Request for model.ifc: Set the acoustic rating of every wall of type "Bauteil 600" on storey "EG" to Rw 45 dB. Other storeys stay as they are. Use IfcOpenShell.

First a look at what the model holds.

```python
import ifcopenshell
import ifcopenshell.util.element

model = ifcopenshell.open("model.ifc")
print(model.schema)
storey = next(s for s in model.by_type("IfcBuildingStorey") if s.Name == "EG")
walls = [e for e in ifcopenshell.util.element.get_decomposition(storey) if e.is_a("IfcWall")]
seen = {}
for e in walls:
    element_type = ifcopenshell.util.element.get_type(e)
    key = (element_type.Name if element_type != e and element_type else None, ifcopenshell.util.element.get_pset(e, "Pset_WallCommon", "AcousticRating"))
    seen[key] = seen.get(key, 0) + 1
for (name, value), count in sorted(seen.items(), key=str):
    print(count, "x", name, "|", value)
```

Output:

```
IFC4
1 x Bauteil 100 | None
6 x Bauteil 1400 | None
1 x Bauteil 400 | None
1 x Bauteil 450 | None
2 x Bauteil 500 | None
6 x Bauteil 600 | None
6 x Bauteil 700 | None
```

```python
import ifcopenshell
import ifcopenshell.api.pset
import ifcopenshell.util.element

model = ifcopenshell.open("model.ifc")

storey = next(s for s in model.by_type("IfcBuildingStorey") if s.Name == "EG")
walls = [e for e in ifcopenshell.util.element.get_decomposition(storey) if e.is_a("IfcWall")]

count = 0
for e in walls:
    element_type = ifcopenshell.util.element.get_type(e)
    if element_type in (None, e) or element_type.Name != "Bauteil 600":
        continue
    # add_pset returns the element's existing set when there is one.
    pset = ifcopenshell.api.pset.add_pset(model, product=e, name="Pset_WallCommon")
    ifcopenshell.api.pset.edit_pset(model, pset=pset, properties={"AcousticRating": "Rw 45 dB"})
    count += 1

print(count, "walls updated")

model.write("model-out.ifc")
```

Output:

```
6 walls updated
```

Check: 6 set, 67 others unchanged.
